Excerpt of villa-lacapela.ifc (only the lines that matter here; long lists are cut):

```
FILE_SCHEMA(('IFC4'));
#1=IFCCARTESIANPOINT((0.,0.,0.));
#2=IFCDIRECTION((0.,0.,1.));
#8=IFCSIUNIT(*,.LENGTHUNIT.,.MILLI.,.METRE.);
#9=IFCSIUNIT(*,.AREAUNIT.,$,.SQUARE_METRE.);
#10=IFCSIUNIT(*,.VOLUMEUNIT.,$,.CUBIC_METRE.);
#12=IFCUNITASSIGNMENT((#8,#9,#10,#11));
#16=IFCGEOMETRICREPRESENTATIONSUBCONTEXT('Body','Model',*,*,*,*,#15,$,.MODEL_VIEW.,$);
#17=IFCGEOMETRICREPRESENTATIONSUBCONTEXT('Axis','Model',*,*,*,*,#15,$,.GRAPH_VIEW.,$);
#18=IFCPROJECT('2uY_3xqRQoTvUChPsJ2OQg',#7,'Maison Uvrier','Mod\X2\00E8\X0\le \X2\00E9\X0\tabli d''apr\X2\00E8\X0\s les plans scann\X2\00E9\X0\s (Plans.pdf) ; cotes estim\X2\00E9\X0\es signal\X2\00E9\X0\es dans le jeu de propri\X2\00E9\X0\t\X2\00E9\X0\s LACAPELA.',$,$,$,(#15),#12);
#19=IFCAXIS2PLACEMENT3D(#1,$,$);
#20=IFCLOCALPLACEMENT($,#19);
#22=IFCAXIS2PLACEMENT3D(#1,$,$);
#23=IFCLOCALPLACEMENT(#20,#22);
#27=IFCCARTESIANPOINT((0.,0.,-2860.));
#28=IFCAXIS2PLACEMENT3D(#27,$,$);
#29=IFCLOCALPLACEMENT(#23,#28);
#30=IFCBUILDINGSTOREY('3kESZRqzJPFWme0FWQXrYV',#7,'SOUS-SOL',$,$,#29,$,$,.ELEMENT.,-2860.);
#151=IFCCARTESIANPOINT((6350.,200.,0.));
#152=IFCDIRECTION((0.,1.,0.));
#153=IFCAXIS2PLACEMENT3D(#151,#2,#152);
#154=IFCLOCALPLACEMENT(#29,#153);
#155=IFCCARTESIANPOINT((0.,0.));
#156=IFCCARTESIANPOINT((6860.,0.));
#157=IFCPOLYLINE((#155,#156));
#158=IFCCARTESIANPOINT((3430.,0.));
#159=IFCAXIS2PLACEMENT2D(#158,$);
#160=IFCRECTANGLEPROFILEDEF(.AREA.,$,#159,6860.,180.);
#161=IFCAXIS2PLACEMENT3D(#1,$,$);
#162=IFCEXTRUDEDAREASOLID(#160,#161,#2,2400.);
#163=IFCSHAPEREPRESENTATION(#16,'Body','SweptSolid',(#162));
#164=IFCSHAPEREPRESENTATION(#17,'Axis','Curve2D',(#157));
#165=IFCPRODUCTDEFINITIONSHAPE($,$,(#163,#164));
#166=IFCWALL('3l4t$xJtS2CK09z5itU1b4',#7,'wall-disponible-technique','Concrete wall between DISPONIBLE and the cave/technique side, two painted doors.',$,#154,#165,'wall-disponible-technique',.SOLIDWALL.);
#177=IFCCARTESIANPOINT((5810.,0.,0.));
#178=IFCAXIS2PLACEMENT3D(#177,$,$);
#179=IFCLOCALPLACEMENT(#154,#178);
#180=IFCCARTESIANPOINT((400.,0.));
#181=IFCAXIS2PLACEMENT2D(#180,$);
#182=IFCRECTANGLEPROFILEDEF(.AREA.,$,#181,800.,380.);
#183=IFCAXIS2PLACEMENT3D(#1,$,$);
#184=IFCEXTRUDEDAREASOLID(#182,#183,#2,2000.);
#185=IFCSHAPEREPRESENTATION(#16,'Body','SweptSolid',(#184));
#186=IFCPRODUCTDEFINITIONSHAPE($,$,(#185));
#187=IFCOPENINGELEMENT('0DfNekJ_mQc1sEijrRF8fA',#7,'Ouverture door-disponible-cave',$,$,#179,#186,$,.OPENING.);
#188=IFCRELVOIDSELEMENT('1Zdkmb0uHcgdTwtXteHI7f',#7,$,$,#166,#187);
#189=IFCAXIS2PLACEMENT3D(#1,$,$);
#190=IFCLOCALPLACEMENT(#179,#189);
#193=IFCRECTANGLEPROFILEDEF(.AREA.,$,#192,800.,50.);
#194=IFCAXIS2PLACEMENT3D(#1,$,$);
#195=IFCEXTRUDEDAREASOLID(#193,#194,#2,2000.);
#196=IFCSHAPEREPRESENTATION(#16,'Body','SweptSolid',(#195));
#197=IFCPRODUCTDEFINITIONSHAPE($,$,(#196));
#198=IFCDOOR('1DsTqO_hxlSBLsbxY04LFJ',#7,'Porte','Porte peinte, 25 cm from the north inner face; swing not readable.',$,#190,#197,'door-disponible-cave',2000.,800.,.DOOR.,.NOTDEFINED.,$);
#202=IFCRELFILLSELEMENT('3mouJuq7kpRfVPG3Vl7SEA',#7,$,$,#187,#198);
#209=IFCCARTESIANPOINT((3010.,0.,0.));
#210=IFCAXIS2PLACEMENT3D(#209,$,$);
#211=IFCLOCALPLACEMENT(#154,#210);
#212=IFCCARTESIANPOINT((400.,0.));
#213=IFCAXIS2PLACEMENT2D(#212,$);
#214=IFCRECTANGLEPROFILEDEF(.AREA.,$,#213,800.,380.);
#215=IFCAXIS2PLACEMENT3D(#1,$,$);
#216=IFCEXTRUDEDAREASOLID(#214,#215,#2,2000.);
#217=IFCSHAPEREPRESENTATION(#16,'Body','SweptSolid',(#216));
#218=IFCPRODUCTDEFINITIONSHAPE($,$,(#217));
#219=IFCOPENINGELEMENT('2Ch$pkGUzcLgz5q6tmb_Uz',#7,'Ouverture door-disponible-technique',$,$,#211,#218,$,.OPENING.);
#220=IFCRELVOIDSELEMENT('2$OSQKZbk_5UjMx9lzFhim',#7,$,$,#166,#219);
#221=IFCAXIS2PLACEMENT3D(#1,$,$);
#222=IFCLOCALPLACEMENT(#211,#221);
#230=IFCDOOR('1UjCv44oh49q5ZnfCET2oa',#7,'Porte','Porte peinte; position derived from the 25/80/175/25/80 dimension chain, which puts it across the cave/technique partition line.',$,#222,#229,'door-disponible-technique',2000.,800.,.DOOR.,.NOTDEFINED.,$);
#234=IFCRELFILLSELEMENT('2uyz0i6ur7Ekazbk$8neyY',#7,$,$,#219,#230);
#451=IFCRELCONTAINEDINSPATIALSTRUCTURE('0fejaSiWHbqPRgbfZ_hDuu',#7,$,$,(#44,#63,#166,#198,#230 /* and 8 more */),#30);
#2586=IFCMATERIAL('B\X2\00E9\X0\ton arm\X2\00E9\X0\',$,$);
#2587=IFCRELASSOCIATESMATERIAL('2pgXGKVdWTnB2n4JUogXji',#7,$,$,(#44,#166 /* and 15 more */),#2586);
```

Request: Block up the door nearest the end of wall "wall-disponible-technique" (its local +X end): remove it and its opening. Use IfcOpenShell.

```python
import ifcopenshell
import ifcopenshell.api.feature
import ifcopenshell.api.root
import ifcopenshell.geom
import ifcopenshell.util.shape

model = ifcopenshell.open("villa-lacapela.ifc")
settings = ifcopenshell.geom.settings()


def volume(element):
    """Net volume in cubic metres, openings subtracted."""
    shape = ifcopenshell.geom.create_shape(settings, element)
    return ifcopenshell.util.shape.get_volume(shape.geometry)


door = model.by_guid("1DsTqO_hxlSBLsbxY04LFJ")
opening = door.FillsVoids[0].RelatingOpeningElement
wall = opening.VoidsElements[0].RelatingBuildingElement
before = volume(wall)

ifcopenshell.api.root.remove_product(model, product=door)
ifcopenshell.api.feature.remove_feature(model, feature=opening)

after = volume(wall)

print(f"wall volume {before:.3f} -> {after:.3f} m3")

model.write("villa-lacapela_v2.ifc")
```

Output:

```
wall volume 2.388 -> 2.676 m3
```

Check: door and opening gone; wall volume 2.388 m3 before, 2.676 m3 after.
